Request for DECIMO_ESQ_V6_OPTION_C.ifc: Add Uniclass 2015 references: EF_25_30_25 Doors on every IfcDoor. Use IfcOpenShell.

First a look at what the model holds.

```python
import ifcopenshell

model = ifcopenshell.open("DECIMO_ESQ_V6_OPTION_C.ifc")
print(model.schema)
print("classifications:", [c.Name for c in model.by_type("IfcClassification")])
for ifc_class in ("IfcDoor", "IfcRoof", "IfcStair", "IfcWall", "IfcWindow"):
    print(ifc_class, len(model.by_type(ifc_class)))
```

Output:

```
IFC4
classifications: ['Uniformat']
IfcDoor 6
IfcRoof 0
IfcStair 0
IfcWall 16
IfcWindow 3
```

```python
import ifcopenshell
import ifcopenshell.api.classification

model = ifcopenshell.open("DECIMO_ESQ_V6_OPTION_C.ifc")

system = ifcopenshell.api.classification.add_classification(model, classification="Uniclass 2015")

codes = {
    "IfcDoor": ("EF_25_30_25", "Doors"),
}
for ifc_class, (code, name) in codes.items():
    products = model.by_type(ifc_class)
    ifcopenshell.api.classification.add_reference(
        model, products=products, classification=system, identification=code, name=name
    )
    print(code, len(products))

model.write("DECIMO_ESQ_V6_OPTION_C_updated.ifc")
```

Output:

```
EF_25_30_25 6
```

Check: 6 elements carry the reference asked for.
